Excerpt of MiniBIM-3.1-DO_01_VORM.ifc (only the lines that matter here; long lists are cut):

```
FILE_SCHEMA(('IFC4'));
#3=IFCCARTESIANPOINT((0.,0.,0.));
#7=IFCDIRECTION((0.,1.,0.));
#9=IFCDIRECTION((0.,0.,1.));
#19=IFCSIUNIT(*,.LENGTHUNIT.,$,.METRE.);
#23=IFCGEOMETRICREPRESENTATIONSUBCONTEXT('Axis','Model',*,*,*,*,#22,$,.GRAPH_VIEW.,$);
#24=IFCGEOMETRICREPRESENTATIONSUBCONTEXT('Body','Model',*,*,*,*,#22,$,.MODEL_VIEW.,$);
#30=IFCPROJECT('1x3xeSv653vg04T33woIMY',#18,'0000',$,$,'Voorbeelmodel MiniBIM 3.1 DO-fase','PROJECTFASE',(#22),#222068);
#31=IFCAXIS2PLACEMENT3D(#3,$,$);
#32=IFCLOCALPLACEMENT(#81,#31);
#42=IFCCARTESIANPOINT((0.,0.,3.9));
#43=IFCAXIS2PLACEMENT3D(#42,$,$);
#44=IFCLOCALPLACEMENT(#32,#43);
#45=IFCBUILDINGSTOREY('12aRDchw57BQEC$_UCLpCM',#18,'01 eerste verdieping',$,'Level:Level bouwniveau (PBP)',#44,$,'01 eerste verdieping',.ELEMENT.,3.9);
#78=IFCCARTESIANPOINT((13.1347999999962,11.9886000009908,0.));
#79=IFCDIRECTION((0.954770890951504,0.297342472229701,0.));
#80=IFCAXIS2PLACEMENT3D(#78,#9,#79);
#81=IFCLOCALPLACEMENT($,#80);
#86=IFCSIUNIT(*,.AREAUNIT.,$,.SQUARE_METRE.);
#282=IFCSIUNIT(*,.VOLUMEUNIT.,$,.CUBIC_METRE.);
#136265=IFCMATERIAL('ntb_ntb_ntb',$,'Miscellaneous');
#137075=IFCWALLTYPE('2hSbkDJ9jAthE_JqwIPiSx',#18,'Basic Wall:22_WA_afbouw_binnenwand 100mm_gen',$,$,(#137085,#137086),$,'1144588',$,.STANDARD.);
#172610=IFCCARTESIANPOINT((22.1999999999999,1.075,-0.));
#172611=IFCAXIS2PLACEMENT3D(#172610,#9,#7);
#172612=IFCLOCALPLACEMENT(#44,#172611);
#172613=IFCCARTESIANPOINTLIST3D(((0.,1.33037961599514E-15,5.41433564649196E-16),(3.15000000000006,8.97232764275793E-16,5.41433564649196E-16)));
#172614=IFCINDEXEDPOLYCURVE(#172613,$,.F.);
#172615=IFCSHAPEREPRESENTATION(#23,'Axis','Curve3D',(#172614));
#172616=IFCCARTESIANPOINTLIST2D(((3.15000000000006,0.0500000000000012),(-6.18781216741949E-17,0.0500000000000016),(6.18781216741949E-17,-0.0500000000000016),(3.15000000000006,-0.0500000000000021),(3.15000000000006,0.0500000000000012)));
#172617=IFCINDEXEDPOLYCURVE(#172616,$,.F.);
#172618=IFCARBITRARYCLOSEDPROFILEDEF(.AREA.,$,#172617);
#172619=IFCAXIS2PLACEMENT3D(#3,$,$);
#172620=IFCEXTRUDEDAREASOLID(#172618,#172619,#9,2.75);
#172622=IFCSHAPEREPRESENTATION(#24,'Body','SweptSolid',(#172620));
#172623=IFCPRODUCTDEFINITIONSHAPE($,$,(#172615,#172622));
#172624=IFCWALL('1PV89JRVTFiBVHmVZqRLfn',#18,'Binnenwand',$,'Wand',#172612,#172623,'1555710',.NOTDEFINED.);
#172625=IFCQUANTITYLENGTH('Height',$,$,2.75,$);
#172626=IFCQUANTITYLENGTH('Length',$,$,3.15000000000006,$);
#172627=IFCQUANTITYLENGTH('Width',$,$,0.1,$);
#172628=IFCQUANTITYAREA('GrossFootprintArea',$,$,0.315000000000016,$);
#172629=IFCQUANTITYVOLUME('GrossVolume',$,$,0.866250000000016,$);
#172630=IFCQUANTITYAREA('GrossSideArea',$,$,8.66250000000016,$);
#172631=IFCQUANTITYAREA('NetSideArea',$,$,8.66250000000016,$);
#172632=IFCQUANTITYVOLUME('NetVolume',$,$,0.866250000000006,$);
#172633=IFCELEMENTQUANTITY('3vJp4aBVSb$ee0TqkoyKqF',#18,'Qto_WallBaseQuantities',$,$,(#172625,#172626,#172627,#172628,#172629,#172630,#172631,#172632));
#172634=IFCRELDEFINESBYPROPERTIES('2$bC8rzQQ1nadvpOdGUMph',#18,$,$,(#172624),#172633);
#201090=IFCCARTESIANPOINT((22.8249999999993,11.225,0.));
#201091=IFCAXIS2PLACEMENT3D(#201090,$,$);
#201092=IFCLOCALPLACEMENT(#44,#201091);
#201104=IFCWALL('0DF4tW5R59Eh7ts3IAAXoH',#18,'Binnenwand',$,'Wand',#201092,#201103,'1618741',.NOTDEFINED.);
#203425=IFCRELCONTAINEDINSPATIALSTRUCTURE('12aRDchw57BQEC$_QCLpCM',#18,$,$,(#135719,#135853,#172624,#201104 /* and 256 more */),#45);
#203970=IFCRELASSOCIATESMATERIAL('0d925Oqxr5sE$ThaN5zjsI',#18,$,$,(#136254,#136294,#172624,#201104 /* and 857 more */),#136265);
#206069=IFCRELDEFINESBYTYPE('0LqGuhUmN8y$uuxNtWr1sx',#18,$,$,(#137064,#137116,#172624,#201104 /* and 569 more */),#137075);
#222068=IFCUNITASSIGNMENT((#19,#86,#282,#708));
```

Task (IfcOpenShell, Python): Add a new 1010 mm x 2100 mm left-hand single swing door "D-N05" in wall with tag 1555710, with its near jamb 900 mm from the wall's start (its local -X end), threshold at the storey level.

```python
import numpy as np
import ifcopenshell
import ifcopenshell.api.feature
import ifcopenshell.api.geometry
import ifcopenshell.api.pset
import ifcopenshell.api.root
import ifcopenshell.api.spatial
import ifcopenshell.geom
import ifcopenshell.util.element
import ifcopenshell.util.placement
import ifcopenshell.util.representation
import ifcopenshell.util.shape
import ifcopenshell.util.unit

model = ifcopenshell.open("MiniBIM-3.1-DO_01_VORM.ifc")
unit_scale = ifcopenshell.util.unit.calculate_unit_scale(model)
area_scale = ifcopenshell.util.unit.calculate_unit_scale(model, "AREAUNIT")
volume_scale = ifcopenshell.util.unit.calculate_unit_scale(model, "VOLUMEUNIT")
settings = ifcopenshell.geom.settings()


def volume(element):
    """Net volume in cubic metres, openings subtracted."""
    shape = ifcopenshell.geom.create_shape(settings, element)
    return ifcopenshell.util.shape.get_volume(shape.geometry)


wall = model.by_guid("1PV89JRVTFiBVHmVZqRLfn")
storey = ifcopenshell.util.element.get_container(wall, ifc_class="IfcBuildingStorey")
context = ifcopenshell.util.representation.get_context(model, "Model", "Body", "MODEL_VIEW")
before = volume(wall)

width, height, from_end, sill = 1.01, 2.1, 0.9, 0.0  # metres

# The wall runs along its own X axis, and the end named is its -X end.
wall_shape = ifcopenshell.geom.create_shape(settings, wall)
x, y, z = ifcopenshell.util.shape.get_vertices(wall_shape.geometry).T
start = x.min() + from_end
face, thickness = float(y.min()), float(y.max() - y.min())
wall_matrix = ifcopenshell.util.placement.get_local_placement(wall.ObjectPlacement)
level = ifcopenshell.util.placement.get_local_placement(storey.ObjectPlacement)[2, 3]


def in_wall(x, y):
    """Placement at x, y metres in the wall's axes, at sill height."""
    matrix = wall_matrix.copy()
    matrix[:, 3] = wall_matrix @ np.array([x / unit_scale, y / unit_scale, 0.0, 1.0])
    matrix[2, 3] = level + sill / unit_scale
    return matrix


# Opening: a box that overshoots both wall faces by 50 mm.
opening = ifcopenshell.api.root.create_entity(model, ifc_class="IfcOpeningElement", predefined_type="OPENING")
box = ifcopenshell.api.geometry.add_wall_representation(
    model, context=context, length=width, height=height, thickness=thickness + 0.1
)
ifcopenshell.api.geometry.assign_representation(model, product=opening, representation=box)
ifcopenshell.api.geometry.edit_object_placement(model, product=opening, matrix=in_wall(start, face - 0.05), is_si=False)
ifcopenshell.api.feature.add_feature(model, feature=opening, element=wall)

door = ifcopenshell.api.root.create_entity(model, ifc_class="IfcDoor", name="D-N05", predefined_type="DOOR")
door.OverallWidth, door.OverallHeight = width / unit_scale, height / unit_scale
door.OperationType = "SINGLE_SWING_LEFT"
body = ifcopenshell.api.geometry.add_door_representation(
    model,
    context=context,
    overall_width=door.OverallWidth,
    overall_height=door.OverallHeight,
    operation_type="SINGLE_SWING_LEFT",
    lining_properties={"LiningDepth": thickness / unit_scale, "ThresholdDepth": thickness / unit_scale},
)
ifcopenshell.api.geometry.assign_representation(model, product=door, representation=body)
ifcopenshell.api.spatial.assign_container(model, products=[door], relating_structure=storey)
ifcopenshell.api.feature.add_filling(model, opening=opening, element=door)

# The lining spans the wall, so the door starts at the wall face.
ifcopenshell.api.geometry.edit_object_placement(model, product=door, matrix=in_wall(start, face), is_si=False)

after = volume(wall)

# Update the wall's stored quantities.
qto = model.by_id(ifcopenshell.util.element.get_pset(wall, "Qto_WallBaseQuantities", should_inherit=False)["id"])
ifcopenshell.api.pset.edit_qto(model, qto=qto, properties={
    "NetSideArea": after / thickness / area_scale,
    "NetVolume": after / volume_scale,
})

print(f"wall volume {before:.3f} -> {after:.3f} m3")

model.write("MiniBIM-3.1-DO_01_VORM_rev.ifc")
```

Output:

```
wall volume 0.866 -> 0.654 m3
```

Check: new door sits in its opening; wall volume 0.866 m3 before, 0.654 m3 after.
